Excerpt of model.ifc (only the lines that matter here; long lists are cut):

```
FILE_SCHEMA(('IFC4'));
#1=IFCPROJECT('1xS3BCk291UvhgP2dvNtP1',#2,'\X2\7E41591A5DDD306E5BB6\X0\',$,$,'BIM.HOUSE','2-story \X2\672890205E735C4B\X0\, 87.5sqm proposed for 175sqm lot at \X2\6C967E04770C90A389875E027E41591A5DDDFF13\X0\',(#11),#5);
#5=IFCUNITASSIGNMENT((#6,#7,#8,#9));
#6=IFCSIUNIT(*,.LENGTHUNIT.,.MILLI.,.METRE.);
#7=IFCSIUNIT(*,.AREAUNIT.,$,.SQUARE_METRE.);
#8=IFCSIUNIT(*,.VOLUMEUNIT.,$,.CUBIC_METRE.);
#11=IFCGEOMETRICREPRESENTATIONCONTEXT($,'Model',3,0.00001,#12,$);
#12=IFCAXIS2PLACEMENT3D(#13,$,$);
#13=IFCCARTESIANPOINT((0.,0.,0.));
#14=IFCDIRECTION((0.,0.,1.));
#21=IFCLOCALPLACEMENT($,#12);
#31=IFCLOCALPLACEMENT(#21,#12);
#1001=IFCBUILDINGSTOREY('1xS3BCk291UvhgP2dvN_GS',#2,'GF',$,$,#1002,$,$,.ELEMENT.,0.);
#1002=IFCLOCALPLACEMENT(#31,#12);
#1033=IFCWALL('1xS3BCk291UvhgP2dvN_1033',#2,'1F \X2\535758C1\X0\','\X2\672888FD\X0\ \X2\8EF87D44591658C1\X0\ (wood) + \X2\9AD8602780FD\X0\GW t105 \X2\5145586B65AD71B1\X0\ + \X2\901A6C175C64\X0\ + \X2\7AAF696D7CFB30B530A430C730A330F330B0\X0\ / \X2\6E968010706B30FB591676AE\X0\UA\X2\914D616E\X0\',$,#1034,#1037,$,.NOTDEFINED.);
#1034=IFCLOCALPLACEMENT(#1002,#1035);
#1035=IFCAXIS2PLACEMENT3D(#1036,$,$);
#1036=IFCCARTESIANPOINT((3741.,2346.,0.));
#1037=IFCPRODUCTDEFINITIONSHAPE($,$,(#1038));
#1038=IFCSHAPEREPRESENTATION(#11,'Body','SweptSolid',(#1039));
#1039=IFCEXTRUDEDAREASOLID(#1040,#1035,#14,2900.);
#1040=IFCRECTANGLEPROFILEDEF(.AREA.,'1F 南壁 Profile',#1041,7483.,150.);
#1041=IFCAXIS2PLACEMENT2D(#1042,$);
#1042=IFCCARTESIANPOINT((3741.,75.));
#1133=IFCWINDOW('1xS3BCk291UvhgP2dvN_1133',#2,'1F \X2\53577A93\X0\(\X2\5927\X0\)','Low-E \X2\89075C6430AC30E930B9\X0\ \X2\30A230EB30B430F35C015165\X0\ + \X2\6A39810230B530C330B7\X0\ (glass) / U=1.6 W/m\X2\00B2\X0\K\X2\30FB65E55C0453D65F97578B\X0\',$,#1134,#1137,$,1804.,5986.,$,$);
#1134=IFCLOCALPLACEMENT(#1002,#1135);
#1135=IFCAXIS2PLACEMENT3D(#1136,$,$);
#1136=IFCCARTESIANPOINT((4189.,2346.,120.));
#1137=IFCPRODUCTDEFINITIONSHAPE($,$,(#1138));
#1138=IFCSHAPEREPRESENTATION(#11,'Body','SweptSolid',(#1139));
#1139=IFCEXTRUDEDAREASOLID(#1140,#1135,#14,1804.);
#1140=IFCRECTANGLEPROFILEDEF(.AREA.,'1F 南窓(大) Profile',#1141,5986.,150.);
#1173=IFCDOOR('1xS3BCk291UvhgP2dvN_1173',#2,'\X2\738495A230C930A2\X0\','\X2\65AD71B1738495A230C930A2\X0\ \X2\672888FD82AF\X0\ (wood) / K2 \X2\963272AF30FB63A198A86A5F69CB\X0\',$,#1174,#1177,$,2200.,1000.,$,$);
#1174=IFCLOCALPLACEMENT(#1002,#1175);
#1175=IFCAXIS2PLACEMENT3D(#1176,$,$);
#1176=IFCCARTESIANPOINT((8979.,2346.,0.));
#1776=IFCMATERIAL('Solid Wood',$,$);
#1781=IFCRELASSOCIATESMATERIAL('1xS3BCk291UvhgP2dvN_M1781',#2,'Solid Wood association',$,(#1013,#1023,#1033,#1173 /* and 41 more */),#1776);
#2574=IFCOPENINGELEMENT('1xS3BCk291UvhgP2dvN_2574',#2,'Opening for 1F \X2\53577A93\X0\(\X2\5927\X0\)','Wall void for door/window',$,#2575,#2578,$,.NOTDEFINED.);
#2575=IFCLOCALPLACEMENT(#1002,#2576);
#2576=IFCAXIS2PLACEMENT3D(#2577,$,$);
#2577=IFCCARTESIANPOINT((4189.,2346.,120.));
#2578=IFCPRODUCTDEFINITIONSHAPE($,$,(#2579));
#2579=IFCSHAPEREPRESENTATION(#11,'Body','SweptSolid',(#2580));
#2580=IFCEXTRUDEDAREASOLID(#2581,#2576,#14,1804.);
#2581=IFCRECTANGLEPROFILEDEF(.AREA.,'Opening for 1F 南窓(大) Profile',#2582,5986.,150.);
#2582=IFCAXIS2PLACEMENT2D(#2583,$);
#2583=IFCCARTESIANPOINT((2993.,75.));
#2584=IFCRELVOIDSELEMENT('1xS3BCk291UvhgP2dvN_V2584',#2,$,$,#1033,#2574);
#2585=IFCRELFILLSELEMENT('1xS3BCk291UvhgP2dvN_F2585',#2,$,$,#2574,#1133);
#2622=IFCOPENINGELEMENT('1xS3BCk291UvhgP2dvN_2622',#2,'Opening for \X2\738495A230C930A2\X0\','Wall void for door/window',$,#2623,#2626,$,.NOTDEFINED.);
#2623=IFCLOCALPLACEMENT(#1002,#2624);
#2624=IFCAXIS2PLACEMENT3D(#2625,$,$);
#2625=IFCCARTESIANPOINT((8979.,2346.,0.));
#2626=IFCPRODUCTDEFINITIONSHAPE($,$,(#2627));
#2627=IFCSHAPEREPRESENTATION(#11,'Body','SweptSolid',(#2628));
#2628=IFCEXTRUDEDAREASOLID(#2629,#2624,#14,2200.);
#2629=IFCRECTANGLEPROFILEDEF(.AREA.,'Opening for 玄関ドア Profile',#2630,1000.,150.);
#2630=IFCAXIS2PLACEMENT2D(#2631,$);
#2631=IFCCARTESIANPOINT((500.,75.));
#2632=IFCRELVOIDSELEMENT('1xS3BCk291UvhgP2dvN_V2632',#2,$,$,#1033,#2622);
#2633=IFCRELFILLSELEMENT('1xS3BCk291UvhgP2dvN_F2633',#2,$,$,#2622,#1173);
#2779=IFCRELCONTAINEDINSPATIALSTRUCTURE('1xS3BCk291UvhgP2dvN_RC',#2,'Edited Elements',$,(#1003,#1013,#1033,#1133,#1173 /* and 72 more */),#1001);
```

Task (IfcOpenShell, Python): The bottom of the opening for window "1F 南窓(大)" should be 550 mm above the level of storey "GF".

```python
import numpy as np
import ifcopenshell
import ifcopenshell.api.geometry
import ifcopenshell.geom
import ifcopenshell.util.element
import ifcopenshell.util.placement
import ifcopenshell.util.shape
import ifcopenshell.util.unit

model = ifcopenshell.open("model.ifc")
unit_scale = ifcopenshell.util.unit.calculate_unit_scale(model)

window = model.by_id(1133)
opening = window.FillsVoids[0].RelatingOpeningElement
storey = ifcopenshell.util.element.get_container(window, ifc_class="IfcBuildingStorey")
level = ifcopenshell.util.placement.get_local_placement(storey.ObjectPlacement)[2, 3]

# The opening's origin need not be at the sill, so measure its lowest point.
shape = ifcopenshell.geom.create_shape(ifcopenshell.geom.settings(), opening)
bottom = ifcopenshell.util.shape.get_shape_bottom_elevation(shape, shape.geometry) / unit_scale
dz = level + 0.55 / unit_scale - bottom

shift = np.array([0.0, 0.0, dz])
# The window is not placed relative to its opening, so move both.
for product in (opening, window):
    matrix = ifcopenshell.util.placement.get_local_placement(product.ObjectPlacement)
    matrix[:3, 3] += shift
    ifcopenshell.api.geometry.edit_object_placement(model, product=product, matrix=matrix, is_si=False)

print(f"moved by {dz * unit_scale:+.3f} m")

model.write("model_edited.ifc")
```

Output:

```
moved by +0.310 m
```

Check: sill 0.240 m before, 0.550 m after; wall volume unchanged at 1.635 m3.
